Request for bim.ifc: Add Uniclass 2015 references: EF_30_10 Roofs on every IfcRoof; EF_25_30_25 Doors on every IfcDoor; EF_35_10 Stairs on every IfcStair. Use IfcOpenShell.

First a look at what the model holds.

```python
import ifcopenshell

model = ifcopenshell.open("bim.ifc")
print(model.schema)
print("classifications:", [c.Name for c in model.by_type("IfcClassification")])
for ifc_class in ("IfcDoor", "IfcRoof", "IfcStair", "IfcWall", "IfcWindow"):
    print(ifc_class, len(model.by_type(ifc_class)))
```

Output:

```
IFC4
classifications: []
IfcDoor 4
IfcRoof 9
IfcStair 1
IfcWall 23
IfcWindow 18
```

```python
import ifcopenshell
import ifcopenshell.api.classification

model = ifcopenshell.open("bim.ifc")

system = ifcopenshell.api.classification.add_classification(model, classification="Uniclass 2015")

codes = {
    "IfcRoof": ("EF_30_10", "Roofs"),
    "IfcDoor": ("EF_25_30_25", "Doors"),
    "IfcStair": ("EF_35_10", "Stairs"),
}
for ifc_class, (code, name) in codes.items():
    products = model.by_type(ifc_class)
    ifcopenshell.api.classification.add_reference(
        model, products=products, classification=system, identification=code, name=name
    )
    print(code, len(products))

model.write("bim_edited.ifc")
```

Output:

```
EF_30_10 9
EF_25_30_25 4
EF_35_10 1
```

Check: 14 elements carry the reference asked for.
